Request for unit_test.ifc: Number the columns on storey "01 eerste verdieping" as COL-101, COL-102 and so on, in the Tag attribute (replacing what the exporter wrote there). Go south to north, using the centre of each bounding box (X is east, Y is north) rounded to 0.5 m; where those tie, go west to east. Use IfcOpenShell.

First a look at what the model holds.

```python
import ifcopenshell
import ifcopenshell.util.element
import ifcopenshell.util.placement

model = ifcopenshell.open("unit_test.ifc")
print(model.schema)
storey = next(s for s in model.by_type("IfcBuildingStorey") if s.Name == "01 eerste verdieping")
columns = [e for e in ifcopenshell.util.element.get_decomposition(storey) if e.is_a("IfcColumn")]
for e in sorted(columns, key=lambda e: e.id()):
    origin = ifcopenshell.util.placement.get_local_placement(e.ObjectPlacement)[:3, 3]
    print(e.id(), e.Tag, e.Name, origin.round(2) + 0.0, sep=" | ")
```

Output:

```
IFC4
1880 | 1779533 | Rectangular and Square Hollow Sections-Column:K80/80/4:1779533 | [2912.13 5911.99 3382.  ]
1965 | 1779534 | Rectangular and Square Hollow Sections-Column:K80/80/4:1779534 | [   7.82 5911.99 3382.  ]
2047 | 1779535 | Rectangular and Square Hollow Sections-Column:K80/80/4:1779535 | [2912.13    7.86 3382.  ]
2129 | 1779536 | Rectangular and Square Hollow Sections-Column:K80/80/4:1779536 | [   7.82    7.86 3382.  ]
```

```python
import ifcopenshell
import ifcopenshell.geom
import ifcopenshell.util.element
import ifcopenshell.util.shape

model = ifcopenshell.open("unit_test.ifc")
settings = ifcopenshell.geom.settings()
settings.set("use-world-coords", True)


def centre(element):
    shape = ifcopenshell.geom.create_shape(settings, element)
    return ifcopenshell.util.shape.get_bbox_centroid(shape.geometry)


storey = next(s for s in model.by_type("IfcBuildingStorey") if s.Name == "01 eerste verdieping")
columns = [e for e in ifcopenshell.util.element.get_decomposition(storey) if e.is_a("IfcColumn")]

# Insertion points can sit at a corner or the storey origin, so sort by the geometry (in metres).
centres = {e: centre(e) for e in columns}
columns.sort(key=lambda e: (round(centres[e][1] / 0.5), centres[e][0]))

for i, e in enumerate(columns, start=1):
    number = f"COL-1{i:02d}"
    e.Tag = number
    print(e.id(), number)

model.write("unit_test_updated.ifc")
```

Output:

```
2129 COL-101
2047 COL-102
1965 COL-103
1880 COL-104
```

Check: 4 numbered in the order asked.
